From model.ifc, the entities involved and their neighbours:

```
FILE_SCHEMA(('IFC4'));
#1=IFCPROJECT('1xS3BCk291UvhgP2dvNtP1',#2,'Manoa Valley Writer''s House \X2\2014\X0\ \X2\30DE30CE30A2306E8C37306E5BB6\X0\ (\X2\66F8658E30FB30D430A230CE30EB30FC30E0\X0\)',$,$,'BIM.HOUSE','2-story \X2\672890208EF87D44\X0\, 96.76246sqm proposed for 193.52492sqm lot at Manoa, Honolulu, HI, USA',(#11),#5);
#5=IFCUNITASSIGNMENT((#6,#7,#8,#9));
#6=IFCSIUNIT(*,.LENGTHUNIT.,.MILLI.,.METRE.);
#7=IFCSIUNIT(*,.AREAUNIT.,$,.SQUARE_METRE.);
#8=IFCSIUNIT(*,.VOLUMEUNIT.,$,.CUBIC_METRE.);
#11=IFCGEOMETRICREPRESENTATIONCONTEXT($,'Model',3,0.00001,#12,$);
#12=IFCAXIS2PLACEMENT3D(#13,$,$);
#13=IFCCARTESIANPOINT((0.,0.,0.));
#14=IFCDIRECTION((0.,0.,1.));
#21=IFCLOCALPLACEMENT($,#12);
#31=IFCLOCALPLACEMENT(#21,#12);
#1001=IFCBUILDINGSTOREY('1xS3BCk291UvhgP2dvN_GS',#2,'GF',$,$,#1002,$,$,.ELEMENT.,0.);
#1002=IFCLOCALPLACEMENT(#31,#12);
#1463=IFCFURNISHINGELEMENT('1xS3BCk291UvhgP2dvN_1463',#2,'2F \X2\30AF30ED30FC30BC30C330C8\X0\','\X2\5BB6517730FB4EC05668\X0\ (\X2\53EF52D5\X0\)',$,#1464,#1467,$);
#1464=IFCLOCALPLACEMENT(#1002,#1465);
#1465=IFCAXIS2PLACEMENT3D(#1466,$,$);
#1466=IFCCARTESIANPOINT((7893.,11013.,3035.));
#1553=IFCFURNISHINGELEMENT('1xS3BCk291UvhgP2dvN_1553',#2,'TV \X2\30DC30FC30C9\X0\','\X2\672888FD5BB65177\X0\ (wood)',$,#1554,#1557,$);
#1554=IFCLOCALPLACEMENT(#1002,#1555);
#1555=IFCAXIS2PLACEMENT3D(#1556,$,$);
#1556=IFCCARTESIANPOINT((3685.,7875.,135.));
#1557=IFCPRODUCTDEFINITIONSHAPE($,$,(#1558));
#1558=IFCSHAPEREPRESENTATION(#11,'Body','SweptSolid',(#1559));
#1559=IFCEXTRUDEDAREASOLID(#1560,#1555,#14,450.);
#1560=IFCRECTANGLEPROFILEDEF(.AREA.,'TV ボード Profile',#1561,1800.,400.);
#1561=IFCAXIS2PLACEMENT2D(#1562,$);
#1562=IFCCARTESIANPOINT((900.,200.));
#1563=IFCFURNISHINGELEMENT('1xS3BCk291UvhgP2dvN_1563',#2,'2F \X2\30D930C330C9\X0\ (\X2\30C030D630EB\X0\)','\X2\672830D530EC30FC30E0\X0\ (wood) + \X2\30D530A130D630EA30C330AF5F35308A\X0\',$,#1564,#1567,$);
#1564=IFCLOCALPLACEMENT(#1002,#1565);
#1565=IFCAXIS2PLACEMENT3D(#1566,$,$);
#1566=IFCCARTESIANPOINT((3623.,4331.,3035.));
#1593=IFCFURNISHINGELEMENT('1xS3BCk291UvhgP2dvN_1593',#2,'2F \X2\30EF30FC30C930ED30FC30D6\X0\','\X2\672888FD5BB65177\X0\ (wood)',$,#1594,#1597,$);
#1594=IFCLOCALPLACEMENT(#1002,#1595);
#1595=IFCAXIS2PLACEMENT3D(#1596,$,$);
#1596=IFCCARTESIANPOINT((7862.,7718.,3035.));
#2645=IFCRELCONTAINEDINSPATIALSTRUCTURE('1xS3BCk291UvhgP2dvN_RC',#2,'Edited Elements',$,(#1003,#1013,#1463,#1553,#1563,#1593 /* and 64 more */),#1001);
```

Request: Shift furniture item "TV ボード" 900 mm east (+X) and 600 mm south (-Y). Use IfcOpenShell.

```python
import ifcopenshell
import ifcopenshell.api.geometry
import ifcopenshell.util.placement

model = ifcopenshell.open("model.ifc")

item = model.by_guid("1xS3BCk291UvhgP2dvN_1553")
matrix = ifcopenshell.util.placement.get_local_placement(item.ObjectPlacement)
matrix[0, 3] += 900.0
matrix[1, 3] -= 600.0
ifcopenshell.api.geometry.edit_object_placement(model, product=item, matrix=matrix, is_si=False)

print(ifcopenshell.util.placement.get_local_placement(item.ObjectPlacement).round(3) + 0.0)

model.write("model_edited.ifc")
```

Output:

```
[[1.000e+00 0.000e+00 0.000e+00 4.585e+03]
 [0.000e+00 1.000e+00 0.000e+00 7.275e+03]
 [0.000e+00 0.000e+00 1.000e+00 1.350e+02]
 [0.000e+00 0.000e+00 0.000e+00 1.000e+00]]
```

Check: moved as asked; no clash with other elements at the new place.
